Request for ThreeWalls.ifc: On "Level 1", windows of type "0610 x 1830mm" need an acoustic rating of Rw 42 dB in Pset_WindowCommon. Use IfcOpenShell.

First a look at what the model holds.

```python
import ifcopenshell
import ifcopenshell.util.element

model = ifcopenshell.open("ThreeWalls.ifc")
print(model.schema)
storey = next(s for s in model.by_type("IfcBuildingStorey") if s.Name == "Level 1")
windows = [e for e in ifcopenshell.util.element.get_decomposition(storey) if e.is_a("IfcWindow")]
seen = {}
for e in windows:
    element_type = ifcopenshell.util.element.get_type(e)
    key = (element_type.Name if element_type != e and element_type else None, ifcopenshell.util.element.get_pset(e, "Pset_WindowCommon", "AcousticRating"))
    seen[key] = seen.get(key, 0) + 1
for (name, value), count in sorted(seen.items(), key=str):
    print(count, "x", name, "|", value)
```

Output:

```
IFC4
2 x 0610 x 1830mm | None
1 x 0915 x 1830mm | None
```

```python
import ifcopenshell
import ifcopenshell.api.pset
import ifcopenshell.util.element

model = ifcopenshell.open("ThreeWalls.ifc")

storey = next(s for s in model.by_type("IfcBuildingStorey") if s.Name == "Level 1")
windows = [e for e in ifcopenshell.util.element.get_decomposition(storey) if e.is_a("IfcWindow")]

count = 0
for e in windows:
    element_type = ifcopenshell.util.element.get_type(e)
    if element_type in (None, e) or element_type.Name != "0610 x 1830mm":
        continue
    # add_pset returns the element's existing set when there is one.
    pset = ifcopenshell.api.pset.add_pset(model, product=e, name="Pset_WindowCommon")
    ifcopenshell.api.pset.edit_pset(model, pset=pset, properties={"AcousticRating": "Rw 42 dB"})
    count += 1

print(count, "windows updated")

model.write("ThreeWalls-out.ifc")
```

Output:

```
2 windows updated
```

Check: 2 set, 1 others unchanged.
